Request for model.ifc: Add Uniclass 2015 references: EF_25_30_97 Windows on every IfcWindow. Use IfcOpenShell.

First a look at what the model holds.

```python
import ifcopenshell

model = ifcopenshell.open("model.ifc")
print(model.schema)
print("classifications:", [c.Name for c in model.by_type("IfcClassification")])
for ifc_class in ("IfcDoor", "IfcRoof", "IfcStair", "IfcWall", "IfcWindow"):
    print(ifc_class, len(model.by_type(ifc_class)))
```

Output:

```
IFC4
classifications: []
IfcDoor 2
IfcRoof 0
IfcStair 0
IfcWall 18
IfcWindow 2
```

```python
import ifcopenshell
import ifcopenshell.api.classification

model = ifcopenshell.open("model.ifc")

system = ifcopenshell.api.classification.add_classification(model, classification="Uniclass 2015")

codes = {
    "IfcWindow": ("EF_25_30_97", "Windows"),
}
for ifc_class, (code, name) in codes.items():
    products = model.by_type(ifc_class)
    ifcopenshell.api.classification.add_reference(
        model, products=products, classification=system, identification=code, name=name
    )
    print(code, len(products))

model.write("model_v2.ifc")
```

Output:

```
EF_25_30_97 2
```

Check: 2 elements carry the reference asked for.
